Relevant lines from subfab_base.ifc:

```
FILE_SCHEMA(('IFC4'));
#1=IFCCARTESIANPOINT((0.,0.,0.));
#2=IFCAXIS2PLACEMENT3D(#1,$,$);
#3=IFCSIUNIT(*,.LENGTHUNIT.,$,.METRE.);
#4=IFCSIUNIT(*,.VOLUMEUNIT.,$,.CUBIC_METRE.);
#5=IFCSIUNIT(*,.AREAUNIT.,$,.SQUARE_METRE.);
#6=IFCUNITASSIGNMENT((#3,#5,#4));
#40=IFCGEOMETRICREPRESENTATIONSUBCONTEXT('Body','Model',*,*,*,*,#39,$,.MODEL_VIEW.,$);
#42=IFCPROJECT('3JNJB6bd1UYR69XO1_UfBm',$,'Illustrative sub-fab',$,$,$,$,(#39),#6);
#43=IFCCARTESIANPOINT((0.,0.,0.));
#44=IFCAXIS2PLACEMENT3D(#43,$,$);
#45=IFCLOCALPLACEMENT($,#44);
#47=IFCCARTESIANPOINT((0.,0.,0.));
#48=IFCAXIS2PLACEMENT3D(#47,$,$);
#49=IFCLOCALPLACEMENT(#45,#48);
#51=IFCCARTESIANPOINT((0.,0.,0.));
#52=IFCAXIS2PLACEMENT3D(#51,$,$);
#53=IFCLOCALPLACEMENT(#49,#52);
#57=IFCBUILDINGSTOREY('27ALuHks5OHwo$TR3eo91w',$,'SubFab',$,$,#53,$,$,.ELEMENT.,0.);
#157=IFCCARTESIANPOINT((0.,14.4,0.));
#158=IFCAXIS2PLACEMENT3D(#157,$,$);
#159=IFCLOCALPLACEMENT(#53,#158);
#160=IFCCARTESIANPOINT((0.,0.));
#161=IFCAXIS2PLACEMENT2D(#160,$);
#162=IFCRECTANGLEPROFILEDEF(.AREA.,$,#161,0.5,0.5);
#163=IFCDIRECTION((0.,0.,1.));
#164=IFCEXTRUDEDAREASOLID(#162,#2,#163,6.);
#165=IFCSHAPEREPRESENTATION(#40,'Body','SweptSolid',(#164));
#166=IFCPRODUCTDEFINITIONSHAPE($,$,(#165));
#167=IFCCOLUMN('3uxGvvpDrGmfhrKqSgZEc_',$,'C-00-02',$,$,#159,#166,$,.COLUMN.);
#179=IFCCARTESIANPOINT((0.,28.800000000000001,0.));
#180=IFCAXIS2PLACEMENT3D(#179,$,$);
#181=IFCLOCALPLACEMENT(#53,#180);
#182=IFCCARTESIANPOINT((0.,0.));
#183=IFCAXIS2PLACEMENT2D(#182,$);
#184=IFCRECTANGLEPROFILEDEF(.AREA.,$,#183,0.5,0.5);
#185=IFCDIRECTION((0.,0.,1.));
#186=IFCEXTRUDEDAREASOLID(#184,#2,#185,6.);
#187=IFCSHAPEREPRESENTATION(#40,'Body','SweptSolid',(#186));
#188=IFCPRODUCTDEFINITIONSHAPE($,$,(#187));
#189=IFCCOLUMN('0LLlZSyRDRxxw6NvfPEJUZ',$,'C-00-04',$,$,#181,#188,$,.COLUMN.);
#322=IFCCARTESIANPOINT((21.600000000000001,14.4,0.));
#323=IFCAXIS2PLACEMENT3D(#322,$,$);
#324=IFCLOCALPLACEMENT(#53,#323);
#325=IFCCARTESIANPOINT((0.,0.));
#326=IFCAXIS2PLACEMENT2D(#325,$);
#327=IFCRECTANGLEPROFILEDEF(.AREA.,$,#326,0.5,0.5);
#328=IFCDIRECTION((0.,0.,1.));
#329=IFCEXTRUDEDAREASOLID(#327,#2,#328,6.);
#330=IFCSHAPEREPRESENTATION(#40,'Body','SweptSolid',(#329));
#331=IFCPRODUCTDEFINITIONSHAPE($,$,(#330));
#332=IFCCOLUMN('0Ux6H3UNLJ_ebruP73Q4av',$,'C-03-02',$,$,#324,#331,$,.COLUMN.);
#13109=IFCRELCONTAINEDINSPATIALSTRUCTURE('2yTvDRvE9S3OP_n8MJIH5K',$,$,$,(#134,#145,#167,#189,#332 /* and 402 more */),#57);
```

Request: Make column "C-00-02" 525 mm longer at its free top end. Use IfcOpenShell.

```python
import ifcopenshell
import ifcopenshell.util.representation
import ifcopenshell.util.unit

model = ifcopenshell.open("subfab_base.ifc")
unit_scale = ifcopenshell.util.unit.calculate_unit_scale(model)

member = model.by_id(167)
change = 0.525 / unit_scale

# The extrusion runs towards the end named, so only its depth changes.
body = ifcopenshell.util.representation.get_representation(member, "Model", "Body")
solid = body.Items[0]
old_length = solid.Depth
solid.Depth += change

print(f"length {old_length:g} -> {solid.Depth:g}")

model.write("subfab_base_updated.ifc")
```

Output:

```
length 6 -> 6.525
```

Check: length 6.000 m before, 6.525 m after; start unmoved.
